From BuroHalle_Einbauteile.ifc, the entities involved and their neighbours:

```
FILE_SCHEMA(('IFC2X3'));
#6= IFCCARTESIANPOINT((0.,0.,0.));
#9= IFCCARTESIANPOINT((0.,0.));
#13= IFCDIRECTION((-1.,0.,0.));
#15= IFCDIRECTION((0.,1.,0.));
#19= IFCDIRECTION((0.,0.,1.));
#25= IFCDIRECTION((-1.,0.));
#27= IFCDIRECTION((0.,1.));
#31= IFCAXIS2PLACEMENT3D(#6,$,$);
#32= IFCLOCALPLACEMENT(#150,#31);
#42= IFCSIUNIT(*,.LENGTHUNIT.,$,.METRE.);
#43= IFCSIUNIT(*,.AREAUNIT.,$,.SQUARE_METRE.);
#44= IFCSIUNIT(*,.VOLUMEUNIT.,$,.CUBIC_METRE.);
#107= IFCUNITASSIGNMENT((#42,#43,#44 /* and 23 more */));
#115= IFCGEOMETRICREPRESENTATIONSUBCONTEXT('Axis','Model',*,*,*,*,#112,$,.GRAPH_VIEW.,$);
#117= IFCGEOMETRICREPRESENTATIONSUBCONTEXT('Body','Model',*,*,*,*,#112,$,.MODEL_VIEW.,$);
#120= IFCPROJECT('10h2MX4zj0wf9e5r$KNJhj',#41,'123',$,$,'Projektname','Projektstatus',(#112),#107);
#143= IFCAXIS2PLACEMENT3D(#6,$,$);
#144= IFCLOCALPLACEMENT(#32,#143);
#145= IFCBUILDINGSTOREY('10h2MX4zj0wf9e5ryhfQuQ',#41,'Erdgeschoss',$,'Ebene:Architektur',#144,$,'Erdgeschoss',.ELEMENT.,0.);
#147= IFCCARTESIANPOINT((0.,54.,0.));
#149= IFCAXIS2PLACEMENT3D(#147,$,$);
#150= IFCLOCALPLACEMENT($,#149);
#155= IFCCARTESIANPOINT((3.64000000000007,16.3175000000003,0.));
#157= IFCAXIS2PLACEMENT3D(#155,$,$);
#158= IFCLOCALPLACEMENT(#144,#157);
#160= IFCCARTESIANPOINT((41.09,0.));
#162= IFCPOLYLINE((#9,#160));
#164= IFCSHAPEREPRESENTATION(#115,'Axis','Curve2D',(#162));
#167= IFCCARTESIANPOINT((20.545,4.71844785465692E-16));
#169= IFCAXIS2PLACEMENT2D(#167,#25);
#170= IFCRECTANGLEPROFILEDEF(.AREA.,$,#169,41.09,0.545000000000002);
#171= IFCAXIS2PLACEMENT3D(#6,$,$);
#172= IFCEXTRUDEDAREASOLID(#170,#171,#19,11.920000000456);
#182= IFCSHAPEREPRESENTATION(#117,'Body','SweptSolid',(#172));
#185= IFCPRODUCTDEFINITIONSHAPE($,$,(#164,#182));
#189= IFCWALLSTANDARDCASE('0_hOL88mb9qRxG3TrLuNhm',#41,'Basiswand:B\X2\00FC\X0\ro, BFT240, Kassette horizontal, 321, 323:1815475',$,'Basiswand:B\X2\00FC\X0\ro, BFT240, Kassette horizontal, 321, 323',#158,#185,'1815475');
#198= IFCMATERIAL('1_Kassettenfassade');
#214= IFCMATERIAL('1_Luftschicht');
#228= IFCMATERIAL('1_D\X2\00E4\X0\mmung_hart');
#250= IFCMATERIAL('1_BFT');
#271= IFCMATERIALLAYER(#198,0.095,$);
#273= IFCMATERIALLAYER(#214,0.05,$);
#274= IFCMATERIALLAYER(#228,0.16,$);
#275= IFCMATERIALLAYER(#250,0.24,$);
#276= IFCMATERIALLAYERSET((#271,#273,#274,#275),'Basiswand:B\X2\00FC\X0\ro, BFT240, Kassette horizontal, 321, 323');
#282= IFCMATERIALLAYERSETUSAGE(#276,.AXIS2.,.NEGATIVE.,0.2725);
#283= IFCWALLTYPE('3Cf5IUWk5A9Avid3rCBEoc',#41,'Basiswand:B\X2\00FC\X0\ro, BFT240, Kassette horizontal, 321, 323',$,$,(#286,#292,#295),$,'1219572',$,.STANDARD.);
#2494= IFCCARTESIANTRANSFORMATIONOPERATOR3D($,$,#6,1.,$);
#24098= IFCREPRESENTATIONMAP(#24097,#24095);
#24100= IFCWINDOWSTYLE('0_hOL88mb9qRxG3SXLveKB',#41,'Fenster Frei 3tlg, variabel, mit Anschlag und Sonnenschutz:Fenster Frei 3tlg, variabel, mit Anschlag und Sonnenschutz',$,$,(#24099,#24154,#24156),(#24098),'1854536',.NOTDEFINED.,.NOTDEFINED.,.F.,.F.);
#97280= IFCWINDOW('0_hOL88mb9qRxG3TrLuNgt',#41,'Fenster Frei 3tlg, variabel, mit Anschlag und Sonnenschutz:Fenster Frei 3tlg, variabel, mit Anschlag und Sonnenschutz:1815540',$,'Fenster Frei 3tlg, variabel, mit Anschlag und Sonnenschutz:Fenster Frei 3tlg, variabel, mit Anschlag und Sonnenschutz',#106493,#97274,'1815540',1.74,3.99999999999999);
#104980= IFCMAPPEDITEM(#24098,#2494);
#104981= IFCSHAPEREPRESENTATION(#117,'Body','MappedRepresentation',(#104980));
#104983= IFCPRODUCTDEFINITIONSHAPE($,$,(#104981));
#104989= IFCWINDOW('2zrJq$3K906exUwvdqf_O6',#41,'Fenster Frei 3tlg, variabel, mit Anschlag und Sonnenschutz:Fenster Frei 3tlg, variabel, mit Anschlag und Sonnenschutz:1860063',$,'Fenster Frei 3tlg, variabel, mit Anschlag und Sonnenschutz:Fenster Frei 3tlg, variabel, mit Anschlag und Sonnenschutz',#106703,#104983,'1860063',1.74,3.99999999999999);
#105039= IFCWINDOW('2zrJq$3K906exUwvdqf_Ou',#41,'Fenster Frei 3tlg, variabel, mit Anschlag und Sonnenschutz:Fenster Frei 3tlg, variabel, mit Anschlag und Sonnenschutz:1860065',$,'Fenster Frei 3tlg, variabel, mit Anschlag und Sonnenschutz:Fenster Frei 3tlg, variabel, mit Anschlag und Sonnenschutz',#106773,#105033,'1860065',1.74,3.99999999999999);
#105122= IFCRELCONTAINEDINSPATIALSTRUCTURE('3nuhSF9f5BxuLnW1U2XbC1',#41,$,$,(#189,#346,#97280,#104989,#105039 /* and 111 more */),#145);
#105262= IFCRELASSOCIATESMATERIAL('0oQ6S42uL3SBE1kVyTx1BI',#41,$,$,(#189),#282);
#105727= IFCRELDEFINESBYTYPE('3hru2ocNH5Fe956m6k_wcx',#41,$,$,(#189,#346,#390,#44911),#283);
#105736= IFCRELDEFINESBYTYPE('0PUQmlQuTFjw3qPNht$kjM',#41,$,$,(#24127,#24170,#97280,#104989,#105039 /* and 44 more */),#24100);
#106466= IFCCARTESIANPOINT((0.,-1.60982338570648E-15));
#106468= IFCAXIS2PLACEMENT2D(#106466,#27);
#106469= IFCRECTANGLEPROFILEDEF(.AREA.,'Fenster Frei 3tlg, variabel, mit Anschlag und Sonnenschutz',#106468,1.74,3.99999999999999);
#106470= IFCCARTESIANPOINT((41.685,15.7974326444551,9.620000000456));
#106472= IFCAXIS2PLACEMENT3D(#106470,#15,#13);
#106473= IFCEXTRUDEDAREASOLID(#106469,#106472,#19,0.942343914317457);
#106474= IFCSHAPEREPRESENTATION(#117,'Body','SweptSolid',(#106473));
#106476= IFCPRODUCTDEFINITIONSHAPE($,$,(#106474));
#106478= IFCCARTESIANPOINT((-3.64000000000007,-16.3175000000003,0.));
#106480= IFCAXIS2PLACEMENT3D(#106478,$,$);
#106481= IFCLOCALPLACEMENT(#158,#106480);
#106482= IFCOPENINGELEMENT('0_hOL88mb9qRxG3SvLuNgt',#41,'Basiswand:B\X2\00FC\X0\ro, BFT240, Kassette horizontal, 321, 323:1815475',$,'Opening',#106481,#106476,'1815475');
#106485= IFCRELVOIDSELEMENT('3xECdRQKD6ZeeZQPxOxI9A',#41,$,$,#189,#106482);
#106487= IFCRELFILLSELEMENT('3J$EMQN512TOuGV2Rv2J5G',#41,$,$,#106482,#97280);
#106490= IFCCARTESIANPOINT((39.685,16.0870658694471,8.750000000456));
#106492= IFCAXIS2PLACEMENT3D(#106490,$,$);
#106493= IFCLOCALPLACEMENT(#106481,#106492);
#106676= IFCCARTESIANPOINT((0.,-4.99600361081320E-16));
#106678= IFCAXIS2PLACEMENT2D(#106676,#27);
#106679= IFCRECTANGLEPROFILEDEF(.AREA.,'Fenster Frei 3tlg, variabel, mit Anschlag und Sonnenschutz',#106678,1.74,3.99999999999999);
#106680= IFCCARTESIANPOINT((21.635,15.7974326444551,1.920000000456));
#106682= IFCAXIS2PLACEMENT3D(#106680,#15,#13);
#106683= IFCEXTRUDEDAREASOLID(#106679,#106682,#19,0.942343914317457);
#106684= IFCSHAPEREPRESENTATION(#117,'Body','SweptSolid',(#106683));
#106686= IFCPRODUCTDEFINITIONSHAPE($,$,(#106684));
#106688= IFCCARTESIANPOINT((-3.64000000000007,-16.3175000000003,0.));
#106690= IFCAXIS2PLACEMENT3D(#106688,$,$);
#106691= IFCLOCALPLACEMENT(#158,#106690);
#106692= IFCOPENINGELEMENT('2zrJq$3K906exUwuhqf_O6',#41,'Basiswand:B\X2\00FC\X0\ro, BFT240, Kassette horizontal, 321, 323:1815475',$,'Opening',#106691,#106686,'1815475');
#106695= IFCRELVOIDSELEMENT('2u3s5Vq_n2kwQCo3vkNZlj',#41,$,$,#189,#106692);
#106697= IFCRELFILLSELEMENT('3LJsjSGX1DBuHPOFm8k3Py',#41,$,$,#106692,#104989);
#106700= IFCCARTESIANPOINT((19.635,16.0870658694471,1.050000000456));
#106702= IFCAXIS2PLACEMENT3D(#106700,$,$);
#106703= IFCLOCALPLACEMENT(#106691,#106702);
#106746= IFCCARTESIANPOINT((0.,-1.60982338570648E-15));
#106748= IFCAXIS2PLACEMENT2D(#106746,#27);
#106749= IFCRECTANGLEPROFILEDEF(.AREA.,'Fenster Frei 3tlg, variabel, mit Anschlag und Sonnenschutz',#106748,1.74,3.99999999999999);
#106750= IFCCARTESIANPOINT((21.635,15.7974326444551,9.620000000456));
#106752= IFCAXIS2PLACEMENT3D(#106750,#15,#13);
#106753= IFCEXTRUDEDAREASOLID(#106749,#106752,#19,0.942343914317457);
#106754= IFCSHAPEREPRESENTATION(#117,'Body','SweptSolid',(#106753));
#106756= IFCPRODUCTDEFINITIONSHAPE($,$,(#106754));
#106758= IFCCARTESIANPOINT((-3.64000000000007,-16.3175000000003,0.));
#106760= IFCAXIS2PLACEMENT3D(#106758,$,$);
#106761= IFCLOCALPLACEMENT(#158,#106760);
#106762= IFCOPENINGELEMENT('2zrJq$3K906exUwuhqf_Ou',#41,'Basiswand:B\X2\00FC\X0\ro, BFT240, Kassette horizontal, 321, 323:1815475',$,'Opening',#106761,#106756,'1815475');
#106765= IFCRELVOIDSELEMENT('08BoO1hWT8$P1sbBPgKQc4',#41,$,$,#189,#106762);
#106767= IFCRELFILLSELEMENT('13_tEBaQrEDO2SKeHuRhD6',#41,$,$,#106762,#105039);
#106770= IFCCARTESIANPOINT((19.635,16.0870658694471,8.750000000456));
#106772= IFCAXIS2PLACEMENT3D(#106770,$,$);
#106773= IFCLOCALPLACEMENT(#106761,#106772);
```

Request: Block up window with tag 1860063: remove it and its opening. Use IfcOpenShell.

```python
import ifcopenshell
import ifcopenshell.api.feature
import ifcopenshell.api.root
import ifcopenshell.geom
import ifcopenshell.util.shape

model = ifcopenshell.open("BuroHalle_Einbauteile.ifc")
settings = ifcopenshell.geom.settings()


def volume(element):
    """Net volume in cubic metres, openings subtracted."""
    shape = ifcopenshell.geom.create_shape(settings, element)
    return ifcopenshell.util.shape.get_volume(shape.geometry)


window = model.by_id(104989)
opening = window.FillsVoids[0].RelatingOpeningElement
wall = opening.VoidsElements[0].RelatingBuildingElement
before = volume(wall)

ifcopenshell.api.root.remove_product(model, product=window)
ifcopenshell.api.feature.remove_feature(model, feature=opening)

after = volume(wall)

print(f"wall volume {before:.3f} -> {after:.3f} m3")

model.write("BuroHalle_Einbauteile-out.ifc")
```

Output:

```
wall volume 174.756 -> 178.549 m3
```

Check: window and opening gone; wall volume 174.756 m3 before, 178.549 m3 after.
